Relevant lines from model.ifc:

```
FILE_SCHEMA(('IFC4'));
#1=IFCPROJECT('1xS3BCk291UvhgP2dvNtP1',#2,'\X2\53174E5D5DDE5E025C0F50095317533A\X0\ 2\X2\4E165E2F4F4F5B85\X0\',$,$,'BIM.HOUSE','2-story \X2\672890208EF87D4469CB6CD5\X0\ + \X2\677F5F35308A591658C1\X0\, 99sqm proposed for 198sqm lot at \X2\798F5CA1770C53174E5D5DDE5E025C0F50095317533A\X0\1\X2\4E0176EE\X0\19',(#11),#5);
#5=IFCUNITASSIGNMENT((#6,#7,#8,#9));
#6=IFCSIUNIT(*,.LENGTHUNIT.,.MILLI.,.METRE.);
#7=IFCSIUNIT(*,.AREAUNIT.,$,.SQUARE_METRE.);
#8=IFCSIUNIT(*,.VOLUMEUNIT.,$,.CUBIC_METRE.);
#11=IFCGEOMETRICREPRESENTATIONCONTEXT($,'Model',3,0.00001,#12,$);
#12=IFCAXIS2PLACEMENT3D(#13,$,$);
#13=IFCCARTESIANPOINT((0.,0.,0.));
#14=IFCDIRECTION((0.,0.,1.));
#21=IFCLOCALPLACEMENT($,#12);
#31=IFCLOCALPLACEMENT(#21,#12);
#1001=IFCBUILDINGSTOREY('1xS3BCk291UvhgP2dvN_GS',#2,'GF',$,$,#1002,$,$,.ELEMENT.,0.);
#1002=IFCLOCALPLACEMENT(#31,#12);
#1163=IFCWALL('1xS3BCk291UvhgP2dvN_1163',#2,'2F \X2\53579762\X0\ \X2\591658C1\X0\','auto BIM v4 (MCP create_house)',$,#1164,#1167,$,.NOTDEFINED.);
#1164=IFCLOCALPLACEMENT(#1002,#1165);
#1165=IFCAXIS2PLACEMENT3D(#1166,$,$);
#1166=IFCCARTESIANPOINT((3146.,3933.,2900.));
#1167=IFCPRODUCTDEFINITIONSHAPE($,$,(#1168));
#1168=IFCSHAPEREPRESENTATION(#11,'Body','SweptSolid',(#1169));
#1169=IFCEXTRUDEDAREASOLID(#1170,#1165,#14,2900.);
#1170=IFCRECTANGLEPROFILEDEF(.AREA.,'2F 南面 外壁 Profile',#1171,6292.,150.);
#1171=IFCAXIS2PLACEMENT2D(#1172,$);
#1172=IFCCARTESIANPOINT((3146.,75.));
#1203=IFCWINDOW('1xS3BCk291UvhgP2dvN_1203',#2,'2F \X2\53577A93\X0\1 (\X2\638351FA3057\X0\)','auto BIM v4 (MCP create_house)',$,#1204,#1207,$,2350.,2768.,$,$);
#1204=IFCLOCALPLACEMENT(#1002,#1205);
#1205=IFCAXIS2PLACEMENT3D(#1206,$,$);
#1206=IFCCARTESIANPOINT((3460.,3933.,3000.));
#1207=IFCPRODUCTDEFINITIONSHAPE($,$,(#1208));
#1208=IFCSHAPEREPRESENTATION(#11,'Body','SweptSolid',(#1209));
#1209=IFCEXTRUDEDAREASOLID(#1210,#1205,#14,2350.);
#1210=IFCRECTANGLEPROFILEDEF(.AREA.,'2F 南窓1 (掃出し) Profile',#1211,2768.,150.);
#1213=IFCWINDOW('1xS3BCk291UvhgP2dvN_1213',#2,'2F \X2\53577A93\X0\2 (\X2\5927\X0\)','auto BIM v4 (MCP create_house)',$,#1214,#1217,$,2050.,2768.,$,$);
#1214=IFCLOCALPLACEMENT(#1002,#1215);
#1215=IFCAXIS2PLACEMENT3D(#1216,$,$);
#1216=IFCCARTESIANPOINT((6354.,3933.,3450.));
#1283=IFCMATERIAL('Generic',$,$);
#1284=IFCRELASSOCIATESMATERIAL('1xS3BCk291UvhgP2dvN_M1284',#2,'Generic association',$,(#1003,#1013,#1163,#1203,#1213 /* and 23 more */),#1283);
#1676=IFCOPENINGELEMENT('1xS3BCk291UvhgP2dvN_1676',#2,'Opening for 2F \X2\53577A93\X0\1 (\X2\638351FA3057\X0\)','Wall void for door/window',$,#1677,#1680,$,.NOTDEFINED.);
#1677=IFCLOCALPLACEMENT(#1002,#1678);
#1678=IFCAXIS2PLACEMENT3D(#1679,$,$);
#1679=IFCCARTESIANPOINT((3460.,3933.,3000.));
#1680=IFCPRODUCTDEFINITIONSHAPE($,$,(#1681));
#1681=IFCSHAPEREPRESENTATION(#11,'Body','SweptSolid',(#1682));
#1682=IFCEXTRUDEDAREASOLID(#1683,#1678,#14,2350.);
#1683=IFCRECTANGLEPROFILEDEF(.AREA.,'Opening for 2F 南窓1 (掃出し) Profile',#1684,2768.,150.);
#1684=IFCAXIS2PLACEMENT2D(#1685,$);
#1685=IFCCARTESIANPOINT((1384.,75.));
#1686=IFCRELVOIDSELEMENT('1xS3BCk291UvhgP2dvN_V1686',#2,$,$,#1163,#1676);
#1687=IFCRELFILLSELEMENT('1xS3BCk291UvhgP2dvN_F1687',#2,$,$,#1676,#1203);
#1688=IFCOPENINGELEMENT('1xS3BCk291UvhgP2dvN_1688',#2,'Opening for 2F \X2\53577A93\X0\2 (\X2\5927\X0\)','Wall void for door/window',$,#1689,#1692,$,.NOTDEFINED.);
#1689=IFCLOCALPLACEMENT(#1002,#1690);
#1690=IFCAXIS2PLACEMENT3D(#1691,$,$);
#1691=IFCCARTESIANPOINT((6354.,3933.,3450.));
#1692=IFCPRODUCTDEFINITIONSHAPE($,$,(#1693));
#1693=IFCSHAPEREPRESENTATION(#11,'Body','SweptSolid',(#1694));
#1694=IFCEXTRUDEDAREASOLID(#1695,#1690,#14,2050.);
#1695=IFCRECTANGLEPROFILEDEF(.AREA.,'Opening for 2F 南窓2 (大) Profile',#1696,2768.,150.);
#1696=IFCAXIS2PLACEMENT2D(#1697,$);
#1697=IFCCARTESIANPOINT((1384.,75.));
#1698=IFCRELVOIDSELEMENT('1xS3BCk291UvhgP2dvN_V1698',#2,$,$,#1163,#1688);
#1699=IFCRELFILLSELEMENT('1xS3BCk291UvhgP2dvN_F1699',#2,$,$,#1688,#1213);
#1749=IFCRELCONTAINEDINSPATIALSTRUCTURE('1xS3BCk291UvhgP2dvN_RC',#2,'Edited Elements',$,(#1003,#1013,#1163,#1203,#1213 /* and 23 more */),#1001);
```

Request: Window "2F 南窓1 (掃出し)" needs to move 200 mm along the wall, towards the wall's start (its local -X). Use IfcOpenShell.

```python
import ifcopenshell
import ifcopenshell.api.geometry
import ifcopenshell.util.placement
import ifcopenshell.util.unit

model = ifcopenshell.open("model.ifc")
unit_scale = ifcopenshell.util.unit.calculate_unit_scale(model)

window = model.by_guid("1xS3BCk291UvhgP2dvN_1203")
opening = window.FillsVoids[0].RelatingOpeningElement
wall = opening.VoidsElements[0].RelatingBuildingElement

wall_matrix = ifcopenshell.util.placement.get_local_placement(wall.ObjectPlacement)
shift = wall_matrix[:3, 0] * -0.2 / unit_scale
before = ifcopenshell.util.placement.get_local_placement(window.ObjectPlacement)[:3, 3].copy()

# The window is not placed relative to its opening, so move both.
for product in (opening, window):
    matrix = ifcopenshell.util.placement.get_local_placement(product.ObjectPlacement)
    matrix[:3, 3] += shift
    ifcopenshell.api.geometry.edit_object_placement(model, product=product, matrix=matrix, is_si=False)

after = ifcopenshell.util.placement.get_local_placement(window.ObjectPlacement)[:3, 3]
print("window moved by", (after - before).round(3) + 0.0)

model.write("model_v2.ifc")
```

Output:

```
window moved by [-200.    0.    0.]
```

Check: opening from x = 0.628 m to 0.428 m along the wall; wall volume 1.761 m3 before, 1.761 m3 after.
